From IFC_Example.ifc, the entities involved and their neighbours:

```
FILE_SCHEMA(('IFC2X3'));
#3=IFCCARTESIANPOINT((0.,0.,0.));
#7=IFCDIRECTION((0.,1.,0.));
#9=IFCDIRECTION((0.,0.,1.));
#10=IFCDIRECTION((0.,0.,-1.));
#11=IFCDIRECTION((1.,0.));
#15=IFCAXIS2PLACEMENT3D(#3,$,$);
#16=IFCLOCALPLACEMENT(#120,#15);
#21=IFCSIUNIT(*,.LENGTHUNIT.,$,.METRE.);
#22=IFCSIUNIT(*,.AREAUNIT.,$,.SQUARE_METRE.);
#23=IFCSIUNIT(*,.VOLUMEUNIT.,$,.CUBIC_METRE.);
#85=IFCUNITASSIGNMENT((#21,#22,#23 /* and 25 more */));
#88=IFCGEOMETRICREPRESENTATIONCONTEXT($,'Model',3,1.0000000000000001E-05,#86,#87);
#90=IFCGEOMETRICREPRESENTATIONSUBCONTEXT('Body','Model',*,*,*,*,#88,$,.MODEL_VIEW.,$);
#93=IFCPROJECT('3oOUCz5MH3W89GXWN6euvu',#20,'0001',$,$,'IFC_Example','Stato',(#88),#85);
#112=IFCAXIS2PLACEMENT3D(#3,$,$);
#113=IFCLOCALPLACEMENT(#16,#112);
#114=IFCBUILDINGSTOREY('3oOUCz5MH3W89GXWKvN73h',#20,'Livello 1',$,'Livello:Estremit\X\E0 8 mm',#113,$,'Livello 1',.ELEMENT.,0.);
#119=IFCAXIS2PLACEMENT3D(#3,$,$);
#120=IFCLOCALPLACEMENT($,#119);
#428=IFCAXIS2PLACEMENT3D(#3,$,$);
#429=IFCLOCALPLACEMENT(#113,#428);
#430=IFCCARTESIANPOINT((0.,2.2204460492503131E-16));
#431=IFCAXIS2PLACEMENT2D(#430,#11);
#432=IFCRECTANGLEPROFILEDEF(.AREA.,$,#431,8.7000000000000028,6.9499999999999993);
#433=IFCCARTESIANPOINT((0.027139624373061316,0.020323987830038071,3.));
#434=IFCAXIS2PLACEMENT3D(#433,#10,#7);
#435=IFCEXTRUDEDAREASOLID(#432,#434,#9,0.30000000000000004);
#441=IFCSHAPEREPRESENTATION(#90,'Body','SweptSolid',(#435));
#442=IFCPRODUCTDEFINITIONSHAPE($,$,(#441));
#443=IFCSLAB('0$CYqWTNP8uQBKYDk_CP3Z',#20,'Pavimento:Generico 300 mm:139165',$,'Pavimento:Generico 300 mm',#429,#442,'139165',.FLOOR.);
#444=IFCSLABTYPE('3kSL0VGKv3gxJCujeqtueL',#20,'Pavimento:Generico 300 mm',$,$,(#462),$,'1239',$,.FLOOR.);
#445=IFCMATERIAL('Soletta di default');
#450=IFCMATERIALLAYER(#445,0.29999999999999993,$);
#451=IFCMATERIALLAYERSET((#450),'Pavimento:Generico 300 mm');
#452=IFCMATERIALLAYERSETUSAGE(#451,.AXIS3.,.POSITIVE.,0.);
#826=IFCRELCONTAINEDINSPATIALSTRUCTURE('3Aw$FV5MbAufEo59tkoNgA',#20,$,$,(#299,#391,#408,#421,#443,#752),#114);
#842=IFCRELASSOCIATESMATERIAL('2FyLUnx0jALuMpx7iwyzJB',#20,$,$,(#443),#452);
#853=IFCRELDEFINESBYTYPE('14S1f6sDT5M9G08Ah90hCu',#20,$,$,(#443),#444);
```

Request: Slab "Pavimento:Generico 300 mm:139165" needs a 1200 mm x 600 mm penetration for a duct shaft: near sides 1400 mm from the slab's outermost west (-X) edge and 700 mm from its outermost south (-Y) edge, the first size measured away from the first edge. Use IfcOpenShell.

```python
import numpy as np
import ifcopenshell
import ifcopenshell.api.feature
import ifcopenshell.api.geometry
import ifcopenshell.api.root
import ifcopenshell.geom
import ifcopenshell.util.placement
import ifcopenshell.util.representation
import ifcopenshell.util.shape
import ifcopenshell.util.unit

model = ifcopenshell.open("IFC_Example.ifc")
unit_scale = ifcopenshell.util.unit.calculate_unit_scale(model)
settings = ifcopenshell.geom.settings()


def volume(element):
    """Net volume in cubic metres, openings subtracted."""
    shape = ifcopenshell.geom.create_shape(settings, element)
    return ifcopenshell.util.shape.get_volume(shape.geometry)


slab = model.by_id(443)
before = volume(slab)

# Extent in the slab's own axes, in metres. The edges named are its -X and -Y sides.
slab_shape = ifcopenshell.geom.create_shape(settings, slab)
vertices = ifcopenshell.util.shape.get_vertices(slab_shape.geometry)
x_min, y_min, bottom = vertices.min(axis=0)
top = vertices[:, 2].max()

opening = ifcopenshell.api.root.create_entity(model, ifc_class="IfcOpeningElement", name="Duct shaft opening")
context = ifcopenshell.util.representation.get_context(model, "Model", "Body", "MODEL_VIEW")
width, depth = 1.2, 0.6
outline = [(0.0, 0.0), (width, 0.0), (width, depth), (0.0, depth), (0.0, 0.0)]
# Overshoot both faces by 50 mm so the cut is clean.
shape = ifcopenshell.api.geometry.add_slab_representation(
    model, context=context, depth=top - bottom + 0.1, polyline=outline
)
ifcopenshell.api.geometry.assign_representation(model, product=opening, representation=shape)

matrix = ifcopenshell.util.placement.get_local_placement(slab.ObjectPlacement)
matrix[:, 3] = matrix @ np.append(np.array([x_min + 1.4, y_min + 0.7, bottom - 0.05]) / unit_scale, 1.0)
ifcopenshell.api.geometry.edit_object_placement(model, product=opening, matrix=matrix, is_si=False)
ifcopenshell.api.feature.add_feature(model, feature=opening, element=slab)

after = volume(slab)

print(f"slab volume {before:.3f} -> {after:.3f} m3")

model.write("IFC_Example_edited.ifc")
```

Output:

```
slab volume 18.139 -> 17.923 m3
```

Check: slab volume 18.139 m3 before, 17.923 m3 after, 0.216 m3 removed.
